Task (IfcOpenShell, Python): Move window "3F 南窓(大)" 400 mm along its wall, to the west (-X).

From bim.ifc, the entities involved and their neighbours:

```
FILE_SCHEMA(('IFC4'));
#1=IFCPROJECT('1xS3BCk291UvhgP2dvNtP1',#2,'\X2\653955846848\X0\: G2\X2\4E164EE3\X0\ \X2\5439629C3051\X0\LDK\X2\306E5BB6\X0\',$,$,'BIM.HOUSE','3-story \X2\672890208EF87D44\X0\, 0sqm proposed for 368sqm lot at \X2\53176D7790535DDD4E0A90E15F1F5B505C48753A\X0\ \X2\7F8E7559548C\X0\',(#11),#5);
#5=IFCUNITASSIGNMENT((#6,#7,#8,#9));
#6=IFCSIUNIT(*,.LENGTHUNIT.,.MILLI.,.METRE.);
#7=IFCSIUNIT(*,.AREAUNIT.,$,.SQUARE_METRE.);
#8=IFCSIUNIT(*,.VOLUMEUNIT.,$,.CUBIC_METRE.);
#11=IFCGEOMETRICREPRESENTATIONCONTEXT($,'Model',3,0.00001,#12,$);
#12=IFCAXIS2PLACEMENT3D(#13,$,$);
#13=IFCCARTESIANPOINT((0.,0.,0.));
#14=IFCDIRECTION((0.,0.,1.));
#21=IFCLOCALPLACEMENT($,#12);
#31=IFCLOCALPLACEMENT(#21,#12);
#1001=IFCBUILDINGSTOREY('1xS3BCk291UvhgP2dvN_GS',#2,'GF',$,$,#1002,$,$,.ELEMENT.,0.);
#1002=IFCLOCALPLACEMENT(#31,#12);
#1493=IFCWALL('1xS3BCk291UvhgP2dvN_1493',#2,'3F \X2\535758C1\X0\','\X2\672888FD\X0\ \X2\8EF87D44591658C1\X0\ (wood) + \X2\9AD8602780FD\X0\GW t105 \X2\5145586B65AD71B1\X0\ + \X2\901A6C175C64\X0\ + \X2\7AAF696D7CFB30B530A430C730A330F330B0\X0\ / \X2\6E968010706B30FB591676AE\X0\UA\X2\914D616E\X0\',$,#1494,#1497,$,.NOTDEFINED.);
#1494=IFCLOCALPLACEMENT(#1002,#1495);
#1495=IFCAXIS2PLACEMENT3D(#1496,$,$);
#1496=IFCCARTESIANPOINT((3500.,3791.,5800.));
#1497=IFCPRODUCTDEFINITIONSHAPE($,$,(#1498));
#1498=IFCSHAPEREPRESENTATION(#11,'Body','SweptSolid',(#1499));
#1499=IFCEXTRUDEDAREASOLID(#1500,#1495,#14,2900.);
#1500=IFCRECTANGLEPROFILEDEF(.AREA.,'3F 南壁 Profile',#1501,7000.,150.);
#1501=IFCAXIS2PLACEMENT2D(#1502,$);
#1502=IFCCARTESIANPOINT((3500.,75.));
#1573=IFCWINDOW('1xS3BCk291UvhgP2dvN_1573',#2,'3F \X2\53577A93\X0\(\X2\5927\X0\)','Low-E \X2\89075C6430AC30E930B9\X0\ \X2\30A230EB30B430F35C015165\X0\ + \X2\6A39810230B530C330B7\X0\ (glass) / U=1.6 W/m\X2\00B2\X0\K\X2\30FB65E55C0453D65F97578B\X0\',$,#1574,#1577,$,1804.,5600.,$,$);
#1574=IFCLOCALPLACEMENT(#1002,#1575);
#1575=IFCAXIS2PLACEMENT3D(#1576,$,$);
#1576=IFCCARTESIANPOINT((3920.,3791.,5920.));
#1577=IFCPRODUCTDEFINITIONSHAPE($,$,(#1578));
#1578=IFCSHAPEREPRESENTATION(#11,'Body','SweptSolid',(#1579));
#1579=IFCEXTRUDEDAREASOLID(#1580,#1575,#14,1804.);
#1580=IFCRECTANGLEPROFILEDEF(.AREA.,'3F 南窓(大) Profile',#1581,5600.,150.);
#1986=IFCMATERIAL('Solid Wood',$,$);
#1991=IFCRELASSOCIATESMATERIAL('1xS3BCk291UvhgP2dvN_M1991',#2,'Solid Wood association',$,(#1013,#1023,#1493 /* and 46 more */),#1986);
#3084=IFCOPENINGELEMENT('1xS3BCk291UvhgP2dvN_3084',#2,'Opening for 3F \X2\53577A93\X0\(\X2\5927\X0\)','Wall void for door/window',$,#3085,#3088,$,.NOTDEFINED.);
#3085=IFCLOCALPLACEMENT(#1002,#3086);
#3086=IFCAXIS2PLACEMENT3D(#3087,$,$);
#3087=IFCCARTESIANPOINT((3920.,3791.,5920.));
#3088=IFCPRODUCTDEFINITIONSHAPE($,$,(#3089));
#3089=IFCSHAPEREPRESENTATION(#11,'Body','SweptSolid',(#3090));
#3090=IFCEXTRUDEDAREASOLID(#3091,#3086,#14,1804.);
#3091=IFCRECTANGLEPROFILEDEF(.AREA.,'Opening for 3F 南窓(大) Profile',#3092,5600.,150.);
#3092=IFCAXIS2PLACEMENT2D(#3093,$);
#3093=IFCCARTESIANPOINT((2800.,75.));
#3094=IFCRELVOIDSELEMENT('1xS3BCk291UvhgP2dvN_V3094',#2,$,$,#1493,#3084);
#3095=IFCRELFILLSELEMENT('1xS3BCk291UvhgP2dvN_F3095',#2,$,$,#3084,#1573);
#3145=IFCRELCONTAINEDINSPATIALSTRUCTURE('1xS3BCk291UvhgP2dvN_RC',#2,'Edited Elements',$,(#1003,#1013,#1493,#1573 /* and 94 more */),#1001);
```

```python
import ifcopenshell
import ifcopenshell.api.geometry
import ifcopenshell.util.placement

model = ifcopenshell.open("bim.ifc")

window = model.by_id(1573)
opening = window.FillsVoids[0].RelatingOpeningElement
wall = opening.VoidsElements[0].RelatingBuildingElement

wall_matrix = ifcopenshell.util.placement.get_local_placement(wall.ObjectPlacement)
shift = wall_matrix[:3, 0] * -400.0
before = ifcopenshell.util.placement.get_local_placement(window.ObjectPlacement)[:3, 3].copy()

# The window is not placed relative to its opening, so move both.
for product in (opening, window):
    matrix = ifcopenshell.util.placement.get_local_placement(product.ObjectPlacement)
    matrix[:3, 3] += shift
    ifcopenshell.api.geometry.edit_object_placement(model, product=product, matrix=matrix, is_si=False)

after = ifcopenshell.util.placement.get_local_placement(window.ObjectPlacement)[:3, 3]
print("window moved by", (after - before).round(3) + 0.0)

model.write("bim-out.ifc")
```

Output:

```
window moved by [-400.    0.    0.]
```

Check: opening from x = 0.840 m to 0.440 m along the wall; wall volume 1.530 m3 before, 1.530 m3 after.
